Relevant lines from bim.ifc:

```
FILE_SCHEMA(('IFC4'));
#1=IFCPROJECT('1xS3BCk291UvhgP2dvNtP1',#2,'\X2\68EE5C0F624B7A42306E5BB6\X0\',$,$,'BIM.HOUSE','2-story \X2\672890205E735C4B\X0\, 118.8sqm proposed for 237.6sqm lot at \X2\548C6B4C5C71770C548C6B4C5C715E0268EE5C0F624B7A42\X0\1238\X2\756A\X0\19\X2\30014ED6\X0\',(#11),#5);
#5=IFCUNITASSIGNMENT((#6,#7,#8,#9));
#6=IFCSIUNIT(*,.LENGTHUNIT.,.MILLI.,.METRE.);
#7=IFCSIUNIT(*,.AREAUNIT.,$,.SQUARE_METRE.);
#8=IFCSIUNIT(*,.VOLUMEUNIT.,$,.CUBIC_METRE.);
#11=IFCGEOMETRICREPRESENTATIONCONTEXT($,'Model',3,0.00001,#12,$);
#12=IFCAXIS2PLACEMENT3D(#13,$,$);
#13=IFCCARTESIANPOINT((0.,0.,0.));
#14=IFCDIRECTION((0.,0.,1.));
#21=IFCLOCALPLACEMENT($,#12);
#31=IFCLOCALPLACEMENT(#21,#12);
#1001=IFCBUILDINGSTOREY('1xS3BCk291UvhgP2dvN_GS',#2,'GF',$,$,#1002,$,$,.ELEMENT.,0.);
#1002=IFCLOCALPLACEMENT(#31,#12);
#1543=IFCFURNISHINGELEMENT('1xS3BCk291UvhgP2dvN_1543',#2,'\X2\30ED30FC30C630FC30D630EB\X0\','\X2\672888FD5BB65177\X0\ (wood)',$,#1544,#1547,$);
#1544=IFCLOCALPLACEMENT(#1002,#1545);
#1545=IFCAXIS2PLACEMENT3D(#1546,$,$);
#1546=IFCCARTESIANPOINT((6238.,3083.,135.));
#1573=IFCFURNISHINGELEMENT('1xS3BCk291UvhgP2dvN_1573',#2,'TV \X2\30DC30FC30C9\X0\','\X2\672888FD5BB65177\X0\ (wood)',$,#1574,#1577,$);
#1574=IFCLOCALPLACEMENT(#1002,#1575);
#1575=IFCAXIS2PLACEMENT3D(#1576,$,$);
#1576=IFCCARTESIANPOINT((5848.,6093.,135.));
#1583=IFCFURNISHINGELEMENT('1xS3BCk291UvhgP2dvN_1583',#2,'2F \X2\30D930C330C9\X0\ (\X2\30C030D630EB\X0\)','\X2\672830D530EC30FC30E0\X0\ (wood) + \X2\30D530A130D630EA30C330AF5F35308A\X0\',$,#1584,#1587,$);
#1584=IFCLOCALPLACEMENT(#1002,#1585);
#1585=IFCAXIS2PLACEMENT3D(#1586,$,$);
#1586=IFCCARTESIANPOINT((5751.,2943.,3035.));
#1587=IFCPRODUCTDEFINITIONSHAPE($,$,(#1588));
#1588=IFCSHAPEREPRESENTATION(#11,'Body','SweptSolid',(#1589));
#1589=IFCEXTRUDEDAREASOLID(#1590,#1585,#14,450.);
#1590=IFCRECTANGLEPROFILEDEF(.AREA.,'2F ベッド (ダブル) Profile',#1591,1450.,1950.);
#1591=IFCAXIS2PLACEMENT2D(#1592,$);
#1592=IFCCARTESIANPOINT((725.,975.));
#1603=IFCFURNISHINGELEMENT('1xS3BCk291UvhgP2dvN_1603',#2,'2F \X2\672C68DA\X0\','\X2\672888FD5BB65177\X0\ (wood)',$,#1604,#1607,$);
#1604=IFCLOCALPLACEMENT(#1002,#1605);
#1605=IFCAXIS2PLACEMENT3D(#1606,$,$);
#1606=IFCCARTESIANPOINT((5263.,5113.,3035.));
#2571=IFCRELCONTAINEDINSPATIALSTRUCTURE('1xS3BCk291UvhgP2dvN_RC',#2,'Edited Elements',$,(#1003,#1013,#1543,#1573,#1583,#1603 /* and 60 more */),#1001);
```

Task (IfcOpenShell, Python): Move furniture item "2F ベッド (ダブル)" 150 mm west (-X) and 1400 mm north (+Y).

```python
import ifcopenshell
import ifcopenshell.api.geometry
import ifcopenshell.util.placement
import ifcopenshell.util.unit

model = ifcopenshell.open("bim.ifc")
unit_scale = ifcopenshell.util.unit.calculate_unit_scale(model)

item = model.by_id(1583)
matrix = ifcopenshell.util.placement.get_local_placement(item.ObjectPlacement)
matrix[0, 3] -= 0.15 / unit_scale
matrix[1, 3] += 1.4 / unit_scale
ifcopenshell.api.geometry.edit_object_placement(model, product=item, matrix=matrix, is_si=False)

print(ifcopenshell.util.placement.get_local_placement(item.ObjectPlacement).round(3) + 0.0)

model.write("bim_edited.ifc")
```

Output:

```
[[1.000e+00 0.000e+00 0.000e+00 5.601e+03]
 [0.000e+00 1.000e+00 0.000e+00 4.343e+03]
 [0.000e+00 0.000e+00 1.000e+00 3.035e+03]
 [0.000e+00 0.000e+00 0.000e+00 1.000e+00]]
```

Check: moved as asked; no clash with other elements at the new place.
